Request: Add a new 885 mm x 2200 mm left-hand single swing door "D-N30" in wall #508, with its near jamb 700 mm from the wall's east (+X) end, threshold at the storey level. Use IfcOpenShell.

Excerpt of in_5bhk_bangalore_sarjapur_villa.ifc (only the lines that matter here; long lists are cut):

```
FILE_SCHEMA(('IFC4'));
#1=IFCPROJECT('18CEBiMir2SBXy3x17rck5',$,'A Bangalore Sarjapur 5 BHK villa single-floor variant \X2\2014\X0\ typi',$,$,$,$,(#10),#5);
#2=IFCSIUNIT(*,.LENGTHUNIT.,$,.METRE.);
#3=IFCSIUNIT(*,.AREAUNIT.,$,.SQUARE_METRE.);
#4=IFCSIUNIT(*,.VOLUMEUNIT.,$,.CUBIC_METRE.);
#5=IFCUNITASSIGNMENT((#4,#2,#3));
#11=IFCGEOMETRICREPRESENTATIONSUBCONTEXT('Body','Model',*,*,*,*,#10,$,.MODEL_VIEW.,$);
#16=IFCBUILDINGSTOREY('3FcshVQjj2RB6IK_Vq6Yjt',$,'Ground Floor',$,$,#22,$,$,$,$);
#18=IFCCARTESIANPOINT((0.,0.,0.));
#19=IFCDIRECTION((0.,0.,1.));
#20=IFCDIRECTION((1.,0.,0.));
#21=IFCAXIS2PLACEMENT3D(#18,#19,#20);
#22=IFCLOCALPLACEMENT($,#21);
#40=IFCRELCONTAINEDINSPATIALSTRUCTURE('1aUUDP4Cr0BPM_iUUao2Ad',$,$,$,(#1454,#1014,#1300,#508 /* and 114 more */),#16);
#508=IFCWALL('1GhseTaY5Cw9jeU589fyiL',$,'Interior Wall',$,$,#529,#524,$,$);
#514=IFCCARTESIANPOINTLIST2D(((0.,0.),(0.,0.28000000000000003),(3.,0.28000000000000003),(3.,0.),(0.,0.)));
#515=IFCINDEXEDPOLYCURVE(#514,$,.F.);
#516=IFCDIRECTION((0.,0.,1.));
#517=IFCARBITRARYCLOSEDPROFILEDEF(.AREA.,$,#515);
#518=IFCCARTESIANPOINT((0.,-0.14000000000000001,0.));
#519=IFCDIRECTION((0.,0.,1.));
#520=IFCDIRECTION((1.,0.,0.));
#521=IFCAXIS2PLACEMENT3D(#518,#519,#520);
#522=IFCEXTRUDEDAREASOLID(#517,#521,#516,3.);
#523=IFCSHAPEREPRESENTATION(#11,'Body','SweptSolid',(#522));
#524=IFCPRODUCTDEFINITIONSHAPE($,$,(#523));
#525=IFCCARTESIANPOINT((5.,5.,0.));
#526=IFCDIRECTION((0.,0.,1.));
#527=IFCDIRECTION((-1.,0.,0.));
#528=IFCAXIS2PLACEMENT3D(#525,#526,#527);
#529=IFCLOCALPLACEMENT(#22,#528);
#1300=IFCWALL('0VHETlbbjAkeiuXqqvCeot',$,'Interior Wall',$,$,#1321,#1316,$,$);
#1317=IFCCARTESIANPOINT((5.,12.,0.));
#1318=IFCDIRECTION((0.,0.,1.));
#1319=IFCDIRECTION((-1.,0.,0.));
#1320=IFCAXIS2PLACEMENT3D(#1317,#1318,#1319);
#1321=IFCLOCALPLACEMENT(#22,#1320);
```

```python
import numpy as np
import ifcopenshell
import ifcopenshell.api.feature
import ifcopenshell.api.geometry
import ifcopenshell.api.root
import ifcopenshell.api.spatial
import ifcopenshell.geom
import ifcopenshell.util.element
import ifcopenshell.util.placement
import ifcopenshell.util.representation
import ifcopenshell.util.shape
import ifcopenshell.util.unit

model = ifcopenshell.open("in_5bhk_bangalore_sarjapur_villa.ifc")
unit_scale = ifcopenshell.util.unit.calculate_unit_scale(model)
settings = ifcopenshell.geom.settings()


def volume(element):
    """Net volume in cubic metres, openings subtracted."""
    shape = ifcopenshell.geom.create_shape(settings, element)
    return ifcopenshell.util.shape.get_volume(shape.geometry)


wall = model.by_guid("1GhseTaY5Cw9jeU589fyiL")
storey = ifcopenshell.util.element.get_container(wall, ifc_class="IfcBuildingStorey")
context = ifcopenshell.util.representation.get_context(model, "Model", "Body", "MODEL_VIEW")
before = volume(wall)

width, height, from_end, sill = 0.885, 2.2, 0.7, 0.0  # metres

# The wall runs along its own X axis, and the end named is its -X end.
wall_shape = ifcopenshell.geom.create_shape(settings, wall)
x, y, z = ifcopenshell.util.shape.get_vertices(wall_shape.geometry).T
start = x.min() + from_end
face, thickness = float(y.min()), float(y.max() - y.min())
wall_matrix = ifcopenshell.util.placement.get_local_placement(wall.ObjectPlacement)
level = ifcopenshell.util.placement.get_local_placement(storey.ObjectPlacement)[2, 3]


def in_wall(x, y):
    """Placement at x, y metres in the wall's axes, at sill height."""
    matrix = wall_matrix.copy()
    matrix[:, 3] = wall_matrix @ np.array([x / unit_scale, y / unit_scale, 0.0, 1.0])
    matrix[2, 3] = level + sill / unit_scale
    return matrix


# Opening: a box that overshoots both wall faces by 50 mm.
opening = ifcopenshell.api.root.create_entity(model, ifc_class="IfcOpeningElement", predefined_type="OPENING")
box = ifcopenshell.api.geometry.add_wall_representation(
    model, context=context, length=width, height=height, thickness=thickness + 0.1
)
ifcopenshell.api.geometry.assign_representation(model, product=opening, representation=box)
ifcopenshell.api.geometry.edit_object_placement(model, product=opening, matrix=in_wall(start, face - 0.05), is_si=False)
ifcopenshell.api.feature.add_feature(model, feature=opening, element=wall)

door = ifcopenshell.api.root.create_entity(model, ifc_class="IfcDoor", name="D-N30", predefined_type="DOOR")
door.OverallWidth, door.OverallHeight = width / unit_scale, height / unit_scale
door.OperationType = "SINGLE_SWING_LEFT"
body = ifcopenshell.api.geometry.add_door_representation(
    model,
    context=context,
    overall_width=door.OverallWidth,
    overall_height=door.OverallHeight,
    operation_type="SINGLE_SWING_LEFT",
    lining_properties={"LiningDepth": thickness / unit_scale, "ThresholdDepth": thickness / unit_scale},
)
ifcopenshell.api.geometry.assign_representation(model, product=door, representation=body)
ifcopenshell.api.spatial.assign_container(model, products=[door], relating_structure=storey)
ifcopenshell.api.feature.add_filling(model, opening=opening, element=door)

# The lining spans the wall, so the door starts at the wall face.
ifcopenshell.api.geometry.edit_object_placement(model, product=door, matrix=in_wall(start, face), is_si=False)

after = volume(wall)

print(f"wall volume {before:.3f} -> {after:.3f} m3")

model.write("in_5bhk_bangalore_sarjapur_villa-out.ifc")
```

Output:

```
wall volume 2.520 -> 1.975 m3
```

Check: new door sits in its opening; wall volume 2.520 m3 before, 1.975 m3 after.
